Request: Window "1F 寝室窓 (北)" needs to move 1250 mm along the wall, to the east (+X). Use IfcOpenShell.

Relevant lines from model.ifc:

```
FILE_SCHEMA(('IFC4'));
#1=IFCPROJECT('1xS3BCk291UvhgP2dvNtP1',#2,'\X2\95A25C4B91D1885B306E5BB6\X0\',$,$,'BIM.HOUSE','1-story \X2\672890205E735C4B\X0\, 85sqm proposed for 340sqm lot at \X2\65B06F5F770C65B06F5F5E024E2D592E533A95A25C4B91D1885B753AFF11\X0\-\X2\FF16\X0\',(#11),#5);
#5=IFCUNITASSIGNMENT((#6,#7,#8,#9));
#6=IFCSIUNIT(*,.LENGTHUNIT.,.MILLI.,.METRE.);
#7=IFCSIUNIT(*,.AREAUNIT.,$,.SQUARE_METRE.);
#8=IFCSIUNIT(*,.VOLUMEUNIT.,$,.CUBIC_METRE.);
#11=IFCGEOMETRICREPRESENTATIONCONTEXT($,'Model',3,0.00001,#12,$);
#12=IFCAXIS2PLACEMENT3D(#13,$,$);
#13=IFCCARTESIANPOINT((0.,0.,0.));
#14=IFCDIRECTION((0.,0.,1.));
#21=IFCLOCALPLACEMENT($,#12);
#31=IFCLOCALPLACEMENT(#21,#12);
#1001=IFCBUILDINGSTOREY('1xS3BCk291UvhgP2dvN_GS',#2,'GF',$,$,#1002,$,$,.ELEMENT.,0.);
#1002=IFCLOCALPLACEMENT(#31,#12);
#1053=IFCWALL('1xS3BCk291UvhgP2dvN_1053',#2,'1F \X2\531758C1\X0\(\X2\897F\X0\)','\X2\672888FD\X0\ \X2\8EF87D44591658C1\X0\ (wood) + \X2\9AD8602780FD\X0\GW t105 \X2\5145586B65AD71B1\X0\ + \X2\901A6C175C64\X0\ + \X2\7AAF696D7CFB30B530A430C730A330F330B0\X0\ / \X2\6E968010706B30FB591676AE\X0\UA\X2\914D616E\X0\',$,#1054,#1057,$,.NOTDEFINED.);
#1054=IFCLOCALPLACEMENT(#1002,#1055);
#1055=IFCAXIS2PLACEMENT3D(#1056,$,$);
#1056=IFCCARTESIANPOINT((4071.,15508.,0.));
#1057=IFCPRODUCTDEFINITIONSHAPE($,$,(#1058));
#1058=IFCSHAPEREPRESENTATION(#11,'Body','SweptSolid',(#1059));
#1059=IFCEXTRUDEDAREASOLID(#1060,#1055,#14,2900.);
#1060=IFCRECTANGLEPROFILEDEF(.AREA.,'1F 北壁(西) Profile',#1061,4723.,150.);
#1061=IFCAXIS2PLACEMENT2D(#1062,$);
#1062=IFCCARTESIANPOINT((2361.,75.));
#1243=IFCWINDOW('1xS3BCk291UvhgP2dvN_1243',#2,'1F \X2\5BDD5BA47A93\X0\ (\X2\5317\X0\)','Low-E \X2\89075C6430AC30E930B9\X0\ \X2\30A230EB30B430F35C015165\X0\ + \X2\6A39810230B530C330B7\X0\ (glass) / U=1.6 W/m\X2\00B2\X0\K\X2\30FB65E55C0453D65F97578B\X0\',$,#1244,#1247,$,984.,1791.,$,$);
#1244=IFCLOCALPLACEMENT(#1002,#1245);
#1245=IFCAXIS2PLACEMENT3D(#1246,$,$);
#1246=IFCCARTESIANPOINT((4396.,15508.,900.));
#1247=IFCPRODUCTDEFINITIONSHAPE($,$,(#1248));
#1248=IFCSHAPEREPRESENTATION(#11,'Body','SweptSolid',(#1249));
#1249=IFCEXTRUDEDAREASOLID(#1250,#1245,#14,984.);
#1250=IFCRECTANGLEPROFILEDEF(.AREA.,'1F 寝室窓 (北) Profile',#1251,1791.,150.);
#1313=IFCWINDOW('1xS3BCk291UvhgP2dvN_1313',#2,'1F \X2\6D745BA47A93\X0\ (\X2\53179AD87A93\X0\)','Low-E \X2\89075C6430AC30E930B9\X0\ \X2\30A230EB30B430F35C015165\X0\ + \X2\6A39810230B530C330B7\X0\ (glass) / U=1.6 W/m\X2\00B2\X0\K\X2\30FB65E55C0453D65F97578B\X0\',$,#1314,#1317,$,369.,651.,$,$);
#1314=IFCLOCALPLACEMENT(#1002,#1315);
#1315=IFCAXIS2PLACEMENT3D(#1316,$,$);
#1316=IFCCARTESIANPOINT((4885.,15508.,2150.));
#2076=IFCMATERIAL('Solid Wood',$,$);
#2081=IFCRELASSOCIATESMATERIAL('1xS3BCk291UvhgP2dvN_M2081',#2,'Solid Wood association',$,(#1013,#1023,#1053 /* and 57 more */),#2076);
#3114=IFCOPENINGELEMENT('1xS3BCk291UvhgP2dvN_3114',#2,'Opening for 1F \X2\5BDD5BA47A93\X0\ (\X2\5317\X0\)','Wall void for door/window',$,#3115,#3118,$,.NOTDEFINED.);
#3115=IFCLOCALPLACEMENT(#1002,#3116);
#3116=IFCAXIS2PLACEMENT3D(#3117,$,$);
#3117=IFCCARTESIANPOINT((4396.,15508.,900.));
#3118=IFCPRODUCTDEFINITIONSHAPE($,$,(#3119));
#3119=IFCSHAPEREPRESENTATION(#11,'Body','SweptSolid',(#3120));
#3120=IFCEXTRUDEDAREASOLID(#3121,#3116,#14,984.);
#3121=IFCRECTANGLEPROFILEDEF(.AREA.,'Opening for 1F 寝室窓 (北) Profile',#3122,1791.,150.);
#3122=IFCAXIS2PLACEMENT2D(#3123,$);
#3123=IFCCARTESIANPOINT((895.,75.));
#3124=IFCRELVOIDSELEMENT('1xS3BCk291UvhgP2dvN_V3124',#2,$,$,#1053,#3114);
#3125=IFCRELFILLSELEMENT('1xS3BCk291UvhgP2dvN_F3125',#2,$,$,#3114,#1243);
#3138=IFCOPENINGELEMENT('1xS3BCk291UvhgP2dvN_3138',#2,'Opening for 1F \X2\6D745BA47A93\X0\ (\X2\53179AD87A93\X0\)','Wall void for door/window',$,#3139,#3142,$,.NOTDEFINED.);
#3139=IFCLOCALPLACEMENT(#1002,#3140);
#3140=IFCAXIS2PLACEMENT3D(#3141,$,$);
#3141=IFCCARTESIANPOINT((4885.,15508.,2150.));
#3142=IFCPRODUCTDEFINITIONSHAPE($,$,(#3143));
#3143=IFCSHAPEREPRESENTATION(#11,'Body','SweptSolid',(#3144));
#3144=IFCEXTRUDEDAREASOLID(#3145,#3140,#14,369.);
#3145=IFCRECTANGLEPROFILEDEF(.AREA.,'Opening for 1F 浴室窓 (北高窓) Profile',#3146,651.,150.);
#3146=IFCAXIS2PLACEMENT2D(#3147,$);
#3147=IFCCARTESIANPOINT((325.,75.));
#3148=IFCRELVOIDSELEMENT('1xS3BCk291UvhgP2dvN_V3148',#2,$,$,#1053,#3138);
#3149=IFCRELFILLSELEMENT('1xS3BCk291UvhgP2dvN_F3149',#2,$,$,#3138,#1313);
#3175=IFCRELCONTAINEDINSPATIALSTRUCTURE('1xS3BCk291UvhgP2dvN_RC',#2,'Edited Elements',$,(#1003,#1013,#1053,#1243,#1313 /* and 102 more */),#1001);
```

```python
import ifcopenshell
import ifcopenshell.api.geometry
import ifcopenshell.util.placement

model = ifcopenshell.open("model.ifc")

window = model.by_id(1243)
opening = window.FillsVoids[0].RelatingOpeningElement
wall = opening.VoidsElements[0].RelatingBuildingElement

wall_matrix = ifcopenshell.util.placement.get_local_placement(wall.ObjectPlacement)
shift = wall_matrix[:3, 0] * 1250.0
before = ifcopenshell.util.placement.get_local_placement(window.ObjectPlacement)[:3, 3].copy()

# The window is not placed relative to its opening, so move both.
for product in (opening, window):
    matrix = ifcopenshell.util.placement.get_local_placement(product.ObjectPlacement)
    matrix[:3, 3] += shift
    ifcopenshell.api.geometry.edit_object_placement(model, product=product, matrix=matrix, is_si=False)

after = ifcopenshell.util.placement.get_local_placement(window.ObjectPlacement)[:3, 3]
print("window moved by", (after - before).round(3) + 0.0)

model.write("model_rev.ifc")
```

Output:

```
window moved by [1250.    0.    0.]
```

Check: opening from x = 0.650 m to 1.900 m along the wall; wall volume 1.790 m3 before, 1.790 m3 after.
